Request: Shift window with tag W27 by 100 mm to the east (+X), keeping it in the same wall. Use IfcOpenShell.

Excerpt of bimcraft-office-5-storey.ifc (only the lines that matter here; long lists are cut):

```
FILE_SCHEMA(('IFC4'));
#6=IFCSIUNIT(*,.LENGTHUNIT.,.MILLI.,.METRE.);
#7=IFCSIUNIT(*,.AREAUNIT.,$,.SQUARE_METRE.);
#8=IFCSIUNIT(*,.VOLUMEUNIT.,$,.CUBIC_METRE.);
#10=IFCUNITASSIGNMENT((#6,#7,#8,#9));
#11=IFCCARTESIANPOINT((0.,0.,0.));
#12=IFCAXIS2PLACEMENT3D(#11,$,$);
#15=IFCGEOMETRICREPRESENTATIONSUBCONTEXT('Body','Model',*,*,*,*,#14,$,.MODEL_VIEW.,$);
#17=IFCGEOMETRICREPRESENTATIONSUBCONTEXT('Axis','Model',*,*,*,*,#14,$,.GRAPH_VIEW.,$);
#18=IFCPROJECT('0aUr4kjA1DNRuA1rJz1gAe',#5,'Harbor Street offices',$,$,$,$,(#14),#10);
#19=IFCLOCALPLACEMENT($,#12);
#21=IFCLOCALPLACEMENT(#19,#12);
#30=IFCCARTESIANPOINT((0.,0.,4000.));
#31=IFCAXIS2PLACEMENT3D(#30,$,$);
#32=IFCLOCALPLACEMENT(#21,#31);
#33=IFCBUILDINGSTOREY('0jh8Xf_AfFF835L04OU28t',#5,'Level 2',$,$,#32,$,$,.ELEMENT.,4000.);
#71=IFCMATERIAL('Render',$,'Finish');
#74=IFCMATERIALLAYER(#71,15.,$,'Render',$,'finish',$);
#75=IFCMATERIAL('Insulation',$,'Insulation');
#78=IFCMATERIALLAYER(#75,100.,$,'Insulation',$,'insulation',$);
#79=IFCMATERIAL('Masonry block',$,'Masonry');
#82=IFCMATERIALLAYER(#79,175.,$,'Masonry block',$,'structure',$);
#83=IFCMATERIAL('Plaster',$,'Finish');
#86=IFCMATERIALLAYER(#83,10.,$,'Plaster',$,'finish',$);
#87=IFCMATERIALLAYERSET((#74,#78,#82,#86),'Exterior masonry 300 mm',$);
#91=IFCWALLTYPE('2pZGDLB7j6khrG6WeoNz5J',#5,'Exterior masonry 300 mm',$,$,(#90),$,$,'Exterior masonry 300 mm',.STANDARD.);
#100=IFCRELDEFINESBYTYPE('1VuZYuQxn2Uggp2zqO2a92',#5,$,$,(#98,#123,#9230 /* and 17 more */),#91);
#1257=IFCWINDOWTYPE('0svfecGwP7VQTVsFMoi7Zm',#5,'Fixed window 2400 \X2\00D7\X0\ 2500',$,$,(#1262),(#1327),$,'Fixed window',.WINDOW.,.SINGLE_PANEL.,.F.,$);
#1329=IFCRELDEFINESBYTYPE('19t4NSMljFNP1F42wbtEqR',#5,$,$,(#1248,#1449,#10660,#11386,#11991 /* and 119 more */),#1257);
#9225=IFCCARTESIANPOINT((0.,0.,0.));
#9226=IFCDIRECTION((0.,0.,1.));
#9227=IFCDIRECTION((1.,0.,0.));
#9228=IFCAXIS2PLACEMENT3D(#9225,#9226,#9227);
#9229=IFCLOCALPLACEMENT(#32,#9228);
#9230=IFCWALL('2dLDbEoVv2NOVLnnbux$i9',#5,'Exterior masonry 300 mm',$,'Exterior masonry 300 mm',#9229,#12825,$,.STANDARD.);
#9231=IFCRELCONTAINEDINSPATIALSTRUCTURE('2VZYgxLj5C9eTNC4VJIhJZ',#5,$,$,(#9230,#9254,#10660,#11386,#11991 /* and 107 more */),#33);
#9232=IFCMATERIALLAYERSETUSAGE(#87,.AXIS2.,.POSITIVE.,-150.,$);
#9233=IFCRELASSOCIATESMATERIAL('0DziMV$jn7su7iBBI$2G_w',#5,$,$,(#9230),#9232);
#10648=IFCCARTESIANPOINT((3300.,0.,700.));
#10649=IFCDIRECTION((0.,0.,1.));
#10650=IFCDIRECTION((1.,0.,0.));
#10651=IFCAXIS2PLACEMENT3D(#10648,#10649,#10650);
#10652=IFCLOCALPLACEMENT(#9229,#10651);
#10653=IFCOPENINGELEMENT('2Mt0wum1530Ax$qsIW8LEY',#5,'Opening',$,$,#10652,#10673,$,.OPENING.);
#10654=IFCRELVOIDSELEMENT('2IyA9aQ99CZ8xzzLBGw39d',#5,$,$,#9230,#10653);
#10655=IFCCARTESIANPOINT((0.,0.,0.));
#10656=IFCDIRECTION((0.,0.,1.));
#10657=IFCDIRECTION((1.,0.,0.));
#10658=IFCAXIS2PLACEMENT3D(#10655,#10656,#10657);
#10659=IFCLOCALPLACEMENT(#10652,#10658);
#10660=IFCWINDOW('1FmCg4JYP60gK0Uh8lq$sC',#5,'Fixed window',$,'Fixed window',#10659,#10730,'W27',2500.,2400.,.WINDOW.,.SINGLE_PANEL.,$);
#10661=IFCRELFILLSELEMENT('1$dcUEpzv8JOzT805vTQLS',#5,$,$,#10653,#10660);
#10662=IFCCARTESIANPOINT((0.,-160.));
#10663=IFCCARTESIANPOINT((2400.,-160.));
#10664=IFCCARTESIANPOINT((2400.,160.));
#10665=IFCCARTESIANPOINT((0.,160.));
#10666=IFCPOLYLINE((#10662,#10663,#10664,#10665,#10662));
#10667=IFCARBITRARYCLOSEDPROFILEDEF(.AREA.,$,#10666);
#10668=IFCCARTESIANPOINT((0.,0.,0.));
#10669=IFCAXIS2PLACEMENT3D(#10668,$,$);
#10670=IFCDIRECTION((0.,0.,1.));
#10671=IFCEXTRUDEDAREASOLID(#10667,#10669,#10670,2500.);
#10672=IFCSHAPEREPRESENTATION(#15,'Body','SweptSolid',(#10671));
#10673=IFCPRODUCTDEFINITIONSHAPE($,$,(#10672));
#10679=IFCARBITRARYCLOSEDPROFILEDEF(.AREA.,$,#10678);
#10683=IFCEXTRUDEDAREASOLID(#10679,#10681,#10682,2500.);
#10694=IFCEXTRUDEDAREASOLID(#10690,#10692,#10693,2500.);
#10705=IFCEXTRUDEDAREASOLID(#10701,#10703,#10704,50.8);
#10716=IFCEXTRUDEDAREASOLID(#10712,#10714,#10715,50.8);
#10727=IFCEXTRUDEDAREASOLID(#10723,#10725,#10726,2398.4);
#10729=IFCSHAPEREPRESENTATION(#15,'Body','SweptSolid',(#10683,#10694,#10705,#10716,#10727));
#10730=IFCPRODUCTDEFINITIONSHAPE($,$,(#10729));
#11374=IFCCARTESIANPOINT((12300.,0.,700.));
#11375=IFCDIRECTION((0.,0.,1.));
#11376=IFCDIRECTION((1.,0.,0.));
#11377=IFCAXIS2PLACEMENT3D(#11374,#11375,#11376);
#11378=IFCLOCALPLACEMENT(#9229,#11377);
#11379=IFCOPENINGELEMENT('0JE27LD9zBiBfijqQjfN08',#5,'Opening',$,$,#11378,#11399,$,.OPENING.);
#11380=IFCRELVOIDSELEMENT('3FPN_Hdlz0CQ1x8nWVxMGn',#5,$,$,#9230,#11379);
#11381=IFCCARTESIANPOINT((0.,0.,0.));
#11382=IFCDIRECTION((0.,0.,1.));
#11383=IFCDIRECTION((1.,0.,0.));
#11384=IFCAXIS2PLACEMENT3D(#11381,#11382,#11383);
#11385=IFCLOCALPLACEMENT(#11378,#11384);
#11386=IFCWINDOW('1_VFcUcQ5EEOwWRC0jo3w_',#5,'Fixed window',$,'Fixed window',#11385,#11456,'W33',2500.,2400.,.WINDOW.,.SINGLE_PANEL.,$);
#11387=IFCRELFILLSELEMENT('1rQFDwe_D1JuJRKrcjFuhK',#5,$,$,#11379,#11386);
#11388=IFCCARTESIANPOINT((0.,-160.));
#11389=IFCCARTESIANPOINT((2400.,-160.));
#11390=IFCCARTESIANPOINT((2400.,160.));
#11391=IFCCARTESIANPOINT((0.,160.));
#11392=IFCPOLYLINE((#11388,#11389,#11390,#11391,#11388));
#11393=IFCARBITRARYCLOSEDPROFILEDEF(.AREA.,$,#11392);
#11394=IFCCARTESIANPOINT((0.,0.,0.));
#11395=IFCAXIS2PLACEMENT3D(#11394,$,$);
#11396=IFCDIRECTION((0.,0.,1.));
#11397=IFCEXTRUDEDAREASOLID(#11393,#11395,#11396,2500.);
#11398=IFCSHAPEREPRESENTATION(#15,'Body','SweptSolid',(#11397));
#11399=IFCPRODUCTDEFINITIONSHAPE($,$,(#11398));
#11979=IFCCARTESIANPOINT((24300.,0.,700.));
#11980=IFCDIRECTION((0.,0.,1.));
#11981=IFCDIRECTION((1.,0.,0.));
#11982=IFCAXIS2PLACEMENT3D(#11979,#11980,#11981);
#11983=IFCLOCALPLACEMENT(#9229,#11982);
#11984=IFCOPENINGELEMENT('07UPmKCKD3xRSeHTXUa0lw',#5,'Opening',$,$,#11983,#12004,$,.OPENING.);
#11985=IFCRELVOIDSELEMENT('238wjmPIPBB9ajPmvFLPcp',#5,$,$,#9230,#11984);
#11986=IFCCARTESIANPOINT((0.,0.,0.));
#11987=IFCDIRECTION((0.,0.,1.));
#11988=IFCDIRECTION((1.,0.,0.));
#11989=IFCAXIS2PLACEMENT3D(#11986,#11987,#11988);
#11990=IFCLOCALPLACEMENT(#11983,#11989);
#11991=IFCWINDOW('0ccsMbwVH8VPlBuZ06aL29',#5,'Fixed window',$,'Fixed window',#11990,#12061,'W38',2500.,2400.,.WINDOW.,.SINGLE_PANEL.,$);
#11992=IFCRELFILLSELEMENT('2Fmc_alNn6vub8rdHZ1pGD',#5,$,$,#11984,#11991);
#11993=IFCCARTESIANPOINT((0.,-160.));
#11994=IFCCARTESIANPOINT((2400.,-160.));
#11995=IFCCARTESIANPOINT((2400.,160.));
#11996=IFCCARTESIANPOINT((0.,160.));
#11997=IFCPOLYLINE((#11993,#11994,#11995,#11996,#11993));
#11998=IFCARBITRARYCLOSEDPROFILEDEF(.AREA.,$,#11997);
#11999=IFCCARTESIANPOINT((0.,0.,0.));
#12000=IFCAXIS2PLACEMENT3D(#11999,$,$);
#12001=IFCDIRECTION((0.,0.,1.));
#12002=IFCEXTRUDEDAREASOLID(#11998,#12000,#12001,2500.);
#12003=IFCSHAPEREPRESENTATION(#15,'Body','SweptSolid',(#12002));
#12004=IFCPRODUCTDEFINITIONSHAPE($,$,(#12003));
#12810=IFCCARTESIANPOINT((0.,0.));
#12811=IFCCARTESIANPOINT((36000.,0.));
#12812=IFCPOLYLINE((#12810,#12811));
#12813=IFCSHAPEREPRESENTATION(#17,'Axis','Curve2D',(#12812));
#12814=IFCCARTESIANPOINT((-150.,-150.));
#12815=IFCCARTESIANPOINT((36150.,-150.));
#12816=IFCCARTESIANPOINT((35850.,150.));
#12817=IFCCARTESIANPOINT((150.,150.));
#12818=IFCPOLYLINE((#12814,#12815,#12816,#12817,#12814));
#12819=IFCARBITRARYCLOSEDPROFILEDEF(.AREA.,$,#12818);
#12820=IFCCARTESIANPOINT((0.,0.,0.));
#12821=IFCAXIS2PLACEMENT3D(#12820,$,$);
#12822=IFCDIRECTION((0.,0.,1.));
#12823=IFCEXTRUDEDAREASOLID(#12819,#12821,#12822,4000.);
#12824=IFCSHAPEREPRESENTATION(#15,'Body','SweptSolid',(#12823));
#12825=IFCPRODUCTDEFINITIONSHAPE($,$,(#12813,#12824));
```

```python
import ifcopenshell
import ifcopenshell.api.geometry
import ifcopenshell.util.placement
import ifcopenshell.util.unit

model = ifcopenshell.open("bimcraft-office-5-storey.ifc")
unit_scale = ifcopenshell.util.unit.calculate_unit_scale(model)

window = model.by_guid("1FmCg4JYP60gK0Uh8lq$sC")
opening = window.FillsVoids[0].RelatingOpeningElement
wall = opening.VoidsElements[0].RelatingBuildingElement

wall_matrix = ifcopenshell.util.placement.get_local_placement(wall.ObjectPlacement)
shift = wall_matrix[:3, 0] * 0.1 / unit_scale
before = ifcopenshell.util.placement.get_local_placement(window.ObjectPlacement)[:3, 3].copy()

# The window is placed relative to its opening, so it follows when the opening moves.
matrix = ifcopenshell.util.placement.get_local_placement(opening.ObjectPlacement)
matrix[:3, 3] += shift
ifcopenshell.api.geometry.edit_object_placement(
    model, product=opening, matrix=matrix, is_si=False, should_transform_children=True
)

after = ifcopenshell.util.placement.get_local_placement(window.ObjectPlacement)[:3, 3]
print("window moved by", (after - before).round(3) + 0.0)

model.write("bimcraft-office-5-storey_v2.ifc")
```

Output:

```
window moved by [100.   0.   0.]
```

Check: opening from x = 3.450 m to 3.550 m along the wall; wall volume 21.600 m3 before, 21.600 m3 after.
